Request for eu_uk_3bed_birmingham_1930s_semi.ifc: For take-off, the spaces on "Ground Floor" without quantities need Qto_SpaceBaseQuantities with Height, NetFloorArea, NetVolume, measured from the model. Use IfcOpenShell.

First a look at what the model holds.

```python
import ifcopenshell
import ifcopenshell.util.element
import ifcopenshell.util.unit

model = ifcopenshell.open("eu_uk_3bed_birmingham_1930s_semi.ifc")
print(model.schema)
for unit_type in ("LENGTHUNIT", "AREAUNIT", "VOLUMEUNIT"):
    print(unit_type, ifcopenshell.util.unit.calculate_unit_scale(model, unit_type))
storey = next(s for s in model.by_type("IfcBuildingStorey") if s.Name == "Ground Floor")
spaces = [e for e in ifcopenshell.util.element.get_decomposition(storey) if e.is_a("IfcSpace")]
for e in sorted(spaces, key=lambda e: e.id()):
    print(e.id(), e.is_a(), e.Name, list(ifcopenshell.util.element.get_psets(e, qtos_only=True)), sep=" | ")
```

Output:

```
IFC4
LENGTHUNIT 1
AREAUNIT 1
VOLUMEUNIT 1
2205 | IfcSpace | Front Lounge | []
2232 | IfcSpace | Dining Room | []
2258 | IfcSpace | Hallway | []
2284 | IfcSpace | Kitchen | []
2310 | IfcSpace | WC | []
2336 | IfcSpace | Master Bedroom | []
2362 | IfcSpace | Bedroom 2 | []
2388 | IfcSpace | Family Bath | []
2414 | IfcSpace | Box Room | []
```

```python
import ifcopenshell
import ifcopenshell.api.pset
import ifcopenshell.geom
import ifcopenshell.util.element
import ifcopenshell.util.shape
import ifcopenshell.util.unit

model = ifcopenshell.open("eu_uk_3bed_birmingham_1930s_semi.ifc")
unit_scale = ifcopenshell.util.unit.calculate_unit_scale(model)
area_scale = ifcopenshell.util.unit.calculate_unit_scale(model, "AREAUNIT")
volume_scale = ifcopenshell.util.unit.calculate_unit_scale(model, "VOLUMEUNIT")
settings = ifcopenshell.geom.settings()

storey = next(s for s in model.by_type("IfcBuildingStorey") if s.Name == "Ground Floor")
spaces = [e for e in ifcopenshell.util.element.get_decomposition(storey) if e.is_a("IfcSpace")]

for e in sorted(spaces, key=lambda e: e.id()):
    if ifcopenshell.util.element.get_psets(e, qtos_only=True, should_inherit=False):
        continue
    # Geometry comes back in metres, in the element's own axes.
    shape = ifcopenshell.geom.create_shape(settings, e)
    values = {
        "Height": ifcopenshell.util.shape.get_z(shape.geometry) / unit_scale,
        "NetFloorArea": ifcopenshell.util.shape.get_footprint_area(shape.geometry) / area_scale,
        "NetVolume": ifcopenshell.util.shape.get_volume(shape.geometry) / volume_scale,
    }
    qto = ifcopenshell.api.pset.add_qto(model, product=e, name="Qto_SpaceBaseQuantities")
    ifcopenshell.api.pset.edit_qto(model, qto=qto, properties=values)
    print(e.id(), {k: round(v, 3) for k, v in values.items()})

model.write("eu_uk_3bed_birmingham_1930s_semi_v2.ifc")
```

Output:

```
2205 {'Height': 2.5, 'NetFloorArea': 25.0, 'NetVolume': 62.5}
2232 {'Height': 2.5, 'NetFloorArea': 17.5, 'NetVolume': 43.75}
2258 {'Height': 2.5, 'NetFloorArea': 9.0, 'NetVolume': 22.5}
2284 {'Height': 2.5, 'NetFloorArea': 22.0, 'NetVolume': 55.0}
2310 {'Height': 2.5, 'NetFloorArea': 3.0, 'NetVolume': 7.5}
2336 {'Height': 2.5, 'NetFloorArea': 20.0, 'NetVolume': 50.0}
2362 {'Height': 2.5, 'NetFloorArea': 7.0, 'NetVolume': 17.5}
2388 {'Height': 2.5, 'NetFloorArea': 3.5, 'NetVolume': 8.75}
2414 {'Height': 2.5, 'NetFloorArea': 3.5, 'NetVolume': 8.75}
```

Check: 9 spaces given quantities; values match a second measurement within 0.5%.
